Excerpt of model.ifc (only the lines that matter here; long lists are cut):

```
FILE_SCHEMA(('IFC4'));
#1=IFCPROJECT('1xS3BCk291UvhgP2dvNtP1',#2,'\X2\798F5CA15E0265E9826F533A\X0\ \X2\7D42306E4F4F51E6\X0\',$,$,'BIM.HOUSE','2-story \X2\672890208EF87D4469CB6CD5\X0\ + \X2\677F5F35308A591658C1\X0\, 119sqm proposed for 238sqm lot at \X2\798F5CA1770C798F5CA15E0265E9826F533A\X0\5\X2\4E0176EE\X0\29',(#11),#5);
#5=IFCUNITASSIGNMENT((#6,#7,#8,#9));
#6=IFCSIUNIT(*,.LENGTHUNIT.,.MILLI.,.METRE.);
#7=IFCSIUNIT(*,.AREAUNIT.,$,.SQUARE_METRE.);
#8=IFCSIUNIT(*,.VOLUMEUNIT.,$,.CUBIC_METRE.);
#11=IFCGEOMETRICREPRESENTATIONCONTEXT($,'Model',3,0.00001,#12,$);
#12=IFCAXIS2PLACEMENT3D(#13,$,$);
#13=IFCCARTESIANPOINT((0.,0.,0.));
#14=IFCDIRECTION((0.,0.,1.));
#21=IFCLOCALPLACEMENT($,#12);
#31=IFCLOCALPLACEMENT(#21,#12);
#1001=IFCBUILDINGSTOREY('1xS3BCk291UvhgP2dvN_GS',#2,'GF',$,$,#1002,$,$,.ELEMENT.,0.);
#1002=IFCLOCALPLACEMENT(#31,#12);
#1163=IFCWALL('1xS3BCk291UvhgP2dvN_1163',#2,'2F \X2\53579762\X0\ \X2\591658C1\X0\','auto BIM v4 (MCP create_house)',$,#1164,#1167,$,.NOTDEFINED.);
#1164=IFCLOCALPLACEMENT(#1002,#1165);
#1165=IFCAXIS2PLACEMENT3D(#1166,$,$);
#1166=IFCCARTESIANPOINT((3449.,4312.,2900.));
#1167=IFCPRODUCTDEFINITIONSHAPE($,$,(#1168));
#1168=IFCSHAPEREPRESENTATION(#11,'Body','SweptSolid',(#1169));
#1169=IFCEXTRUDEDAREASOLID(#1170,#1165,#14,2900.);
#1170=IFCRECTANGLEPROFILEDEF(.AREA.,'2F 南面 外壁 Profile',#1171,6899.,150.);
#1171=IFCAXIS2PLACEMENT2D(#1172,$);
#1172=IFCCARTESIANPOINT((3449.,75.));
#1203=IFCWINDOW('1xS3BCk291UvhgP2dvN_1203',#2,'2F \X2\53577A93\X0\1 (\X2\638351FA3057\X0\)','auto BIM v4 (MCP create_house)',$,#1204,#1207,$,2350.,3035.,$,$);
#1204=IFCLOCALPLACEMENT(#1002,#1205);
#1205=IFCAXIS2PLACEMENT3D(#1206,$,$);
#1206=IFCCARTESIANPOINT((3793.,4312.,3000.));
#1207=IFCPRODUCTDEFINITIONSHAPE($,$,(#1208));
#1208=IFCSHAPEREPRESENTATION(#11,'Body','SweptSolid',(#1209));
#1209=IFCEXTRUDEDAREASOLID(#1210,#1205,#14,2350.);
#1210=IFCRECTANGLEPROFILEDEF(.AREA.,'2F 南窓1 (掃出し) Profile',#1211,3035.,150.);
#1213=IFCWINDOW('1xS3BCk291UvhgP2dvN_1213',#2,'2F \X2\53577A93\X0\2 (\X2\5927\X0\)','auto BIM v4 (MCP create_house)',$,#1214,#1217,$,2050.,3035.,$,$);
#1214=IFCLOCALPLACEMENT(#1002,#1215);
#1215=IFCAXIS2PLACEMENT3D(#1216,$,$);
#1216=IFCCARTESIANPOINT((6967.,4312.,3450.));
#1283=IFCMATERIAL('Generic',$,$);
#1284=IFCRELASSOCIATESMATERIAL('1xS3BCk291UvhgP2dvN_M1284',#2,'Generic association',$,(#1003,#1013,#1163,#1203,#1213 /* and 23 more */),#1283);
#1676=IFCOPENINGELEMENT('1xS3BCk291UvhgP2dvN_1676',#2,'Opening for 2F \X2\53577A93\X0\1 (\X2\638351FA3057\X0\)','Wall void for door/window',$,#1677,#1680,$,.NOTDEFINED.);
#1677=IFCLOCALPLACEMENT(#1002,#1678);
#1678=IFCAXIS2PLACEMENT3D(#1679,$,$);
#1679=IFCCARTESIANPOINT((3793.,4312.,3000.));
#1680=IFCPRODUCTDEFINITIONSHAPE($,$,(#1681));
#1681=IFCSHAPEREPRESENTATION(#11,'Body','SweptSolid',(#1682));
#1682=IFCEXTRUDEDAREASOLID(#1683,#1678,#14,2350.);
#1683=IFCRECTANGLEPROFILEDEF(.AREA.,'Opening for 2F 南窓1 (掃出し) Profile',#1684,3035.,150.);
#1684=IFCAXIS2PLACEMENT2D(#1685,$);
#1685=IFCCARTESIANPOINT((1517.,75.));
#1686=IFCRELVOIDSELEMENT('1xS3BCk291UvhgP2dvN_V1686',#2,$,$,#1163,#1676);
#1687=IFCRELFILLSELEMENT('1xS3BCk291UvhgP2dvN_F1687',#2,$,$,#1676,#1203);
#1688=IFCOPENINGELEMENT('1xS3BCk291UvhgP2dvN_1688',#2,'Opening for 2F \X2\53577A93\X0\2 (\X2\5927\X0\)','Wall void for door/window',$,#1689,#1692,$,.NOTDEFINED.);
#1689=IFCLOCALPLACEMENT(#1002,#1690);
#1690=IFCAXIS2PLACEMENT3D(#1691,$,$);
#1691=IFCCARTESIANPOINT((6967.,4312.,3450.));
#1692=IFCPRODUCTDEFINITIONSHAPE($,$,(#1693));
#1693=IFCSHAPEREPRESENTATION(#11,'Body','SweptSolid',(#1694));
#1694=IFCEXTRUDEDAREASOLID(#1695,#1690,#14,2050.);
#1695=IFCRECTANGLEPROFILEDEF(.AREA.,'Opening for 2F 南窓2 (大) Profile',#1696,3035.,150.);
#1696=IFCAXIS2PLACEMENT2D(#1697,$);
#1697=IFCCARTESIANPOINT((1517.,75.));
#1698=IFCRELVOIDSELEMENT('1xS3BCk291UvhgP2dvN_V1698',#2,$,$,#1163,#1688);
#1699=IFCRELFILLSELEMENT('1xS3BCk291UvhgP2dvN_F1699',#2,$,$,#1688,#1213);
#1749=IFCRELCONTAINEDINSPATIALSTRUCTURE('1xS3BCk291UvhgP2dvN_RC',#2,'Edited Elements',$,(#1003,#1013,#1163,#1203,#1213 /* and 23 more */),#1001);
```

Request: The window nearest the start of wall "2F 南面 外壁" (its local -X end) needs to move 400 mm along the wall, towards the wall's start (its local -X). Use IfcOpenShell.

```python
import ifcopenshell
import ifcopenshell.api.geometry
import ifcopenshell.util.placement
import ifcopenshell.util.unit

model = ifcopenshell.open("model.ifc")
unit_scale = ifcopenshell.util.unit.calculate_unit_scale(model)

window = model.by_id(1203)
opening = window.FillsVoids[0].RelatingOpeningElement
wall = opening.VoidsElements[0].RelatingBuildingElement

wall_matrix = ifcopenshell.util.placement.get_local_placement(wall.ObjectPlacement)
shift = wall_matrix[:3, 0] * -0.4 / unit_scale
before = ifcopenshell.util.placement.get_local_placement(window.ObjectPlacement)[:3, 3].copy()

# The window is not placed relative to its opening, so move both.
for product in (opening, window):
    matrix = ifcopenshell.util.placement.get_local_placement(product.ObjectPlacement)
    matrix[:3, 3] += shift
    ifcopenshell.api.geometry.edit_object_placement(model, product=product, matrix=matrix, is_si=False)

after = ifcopenshell.util.placement.get_local_placement(window.ObjectPlacement)[:3, 3]
print("window moved by", (after - before).round(3) + 0.0)

model.write("model_edited.ifc")
```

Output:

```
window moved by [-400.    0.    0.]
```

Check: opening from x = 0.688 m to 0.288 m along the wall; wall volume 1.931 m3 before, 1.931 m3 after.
